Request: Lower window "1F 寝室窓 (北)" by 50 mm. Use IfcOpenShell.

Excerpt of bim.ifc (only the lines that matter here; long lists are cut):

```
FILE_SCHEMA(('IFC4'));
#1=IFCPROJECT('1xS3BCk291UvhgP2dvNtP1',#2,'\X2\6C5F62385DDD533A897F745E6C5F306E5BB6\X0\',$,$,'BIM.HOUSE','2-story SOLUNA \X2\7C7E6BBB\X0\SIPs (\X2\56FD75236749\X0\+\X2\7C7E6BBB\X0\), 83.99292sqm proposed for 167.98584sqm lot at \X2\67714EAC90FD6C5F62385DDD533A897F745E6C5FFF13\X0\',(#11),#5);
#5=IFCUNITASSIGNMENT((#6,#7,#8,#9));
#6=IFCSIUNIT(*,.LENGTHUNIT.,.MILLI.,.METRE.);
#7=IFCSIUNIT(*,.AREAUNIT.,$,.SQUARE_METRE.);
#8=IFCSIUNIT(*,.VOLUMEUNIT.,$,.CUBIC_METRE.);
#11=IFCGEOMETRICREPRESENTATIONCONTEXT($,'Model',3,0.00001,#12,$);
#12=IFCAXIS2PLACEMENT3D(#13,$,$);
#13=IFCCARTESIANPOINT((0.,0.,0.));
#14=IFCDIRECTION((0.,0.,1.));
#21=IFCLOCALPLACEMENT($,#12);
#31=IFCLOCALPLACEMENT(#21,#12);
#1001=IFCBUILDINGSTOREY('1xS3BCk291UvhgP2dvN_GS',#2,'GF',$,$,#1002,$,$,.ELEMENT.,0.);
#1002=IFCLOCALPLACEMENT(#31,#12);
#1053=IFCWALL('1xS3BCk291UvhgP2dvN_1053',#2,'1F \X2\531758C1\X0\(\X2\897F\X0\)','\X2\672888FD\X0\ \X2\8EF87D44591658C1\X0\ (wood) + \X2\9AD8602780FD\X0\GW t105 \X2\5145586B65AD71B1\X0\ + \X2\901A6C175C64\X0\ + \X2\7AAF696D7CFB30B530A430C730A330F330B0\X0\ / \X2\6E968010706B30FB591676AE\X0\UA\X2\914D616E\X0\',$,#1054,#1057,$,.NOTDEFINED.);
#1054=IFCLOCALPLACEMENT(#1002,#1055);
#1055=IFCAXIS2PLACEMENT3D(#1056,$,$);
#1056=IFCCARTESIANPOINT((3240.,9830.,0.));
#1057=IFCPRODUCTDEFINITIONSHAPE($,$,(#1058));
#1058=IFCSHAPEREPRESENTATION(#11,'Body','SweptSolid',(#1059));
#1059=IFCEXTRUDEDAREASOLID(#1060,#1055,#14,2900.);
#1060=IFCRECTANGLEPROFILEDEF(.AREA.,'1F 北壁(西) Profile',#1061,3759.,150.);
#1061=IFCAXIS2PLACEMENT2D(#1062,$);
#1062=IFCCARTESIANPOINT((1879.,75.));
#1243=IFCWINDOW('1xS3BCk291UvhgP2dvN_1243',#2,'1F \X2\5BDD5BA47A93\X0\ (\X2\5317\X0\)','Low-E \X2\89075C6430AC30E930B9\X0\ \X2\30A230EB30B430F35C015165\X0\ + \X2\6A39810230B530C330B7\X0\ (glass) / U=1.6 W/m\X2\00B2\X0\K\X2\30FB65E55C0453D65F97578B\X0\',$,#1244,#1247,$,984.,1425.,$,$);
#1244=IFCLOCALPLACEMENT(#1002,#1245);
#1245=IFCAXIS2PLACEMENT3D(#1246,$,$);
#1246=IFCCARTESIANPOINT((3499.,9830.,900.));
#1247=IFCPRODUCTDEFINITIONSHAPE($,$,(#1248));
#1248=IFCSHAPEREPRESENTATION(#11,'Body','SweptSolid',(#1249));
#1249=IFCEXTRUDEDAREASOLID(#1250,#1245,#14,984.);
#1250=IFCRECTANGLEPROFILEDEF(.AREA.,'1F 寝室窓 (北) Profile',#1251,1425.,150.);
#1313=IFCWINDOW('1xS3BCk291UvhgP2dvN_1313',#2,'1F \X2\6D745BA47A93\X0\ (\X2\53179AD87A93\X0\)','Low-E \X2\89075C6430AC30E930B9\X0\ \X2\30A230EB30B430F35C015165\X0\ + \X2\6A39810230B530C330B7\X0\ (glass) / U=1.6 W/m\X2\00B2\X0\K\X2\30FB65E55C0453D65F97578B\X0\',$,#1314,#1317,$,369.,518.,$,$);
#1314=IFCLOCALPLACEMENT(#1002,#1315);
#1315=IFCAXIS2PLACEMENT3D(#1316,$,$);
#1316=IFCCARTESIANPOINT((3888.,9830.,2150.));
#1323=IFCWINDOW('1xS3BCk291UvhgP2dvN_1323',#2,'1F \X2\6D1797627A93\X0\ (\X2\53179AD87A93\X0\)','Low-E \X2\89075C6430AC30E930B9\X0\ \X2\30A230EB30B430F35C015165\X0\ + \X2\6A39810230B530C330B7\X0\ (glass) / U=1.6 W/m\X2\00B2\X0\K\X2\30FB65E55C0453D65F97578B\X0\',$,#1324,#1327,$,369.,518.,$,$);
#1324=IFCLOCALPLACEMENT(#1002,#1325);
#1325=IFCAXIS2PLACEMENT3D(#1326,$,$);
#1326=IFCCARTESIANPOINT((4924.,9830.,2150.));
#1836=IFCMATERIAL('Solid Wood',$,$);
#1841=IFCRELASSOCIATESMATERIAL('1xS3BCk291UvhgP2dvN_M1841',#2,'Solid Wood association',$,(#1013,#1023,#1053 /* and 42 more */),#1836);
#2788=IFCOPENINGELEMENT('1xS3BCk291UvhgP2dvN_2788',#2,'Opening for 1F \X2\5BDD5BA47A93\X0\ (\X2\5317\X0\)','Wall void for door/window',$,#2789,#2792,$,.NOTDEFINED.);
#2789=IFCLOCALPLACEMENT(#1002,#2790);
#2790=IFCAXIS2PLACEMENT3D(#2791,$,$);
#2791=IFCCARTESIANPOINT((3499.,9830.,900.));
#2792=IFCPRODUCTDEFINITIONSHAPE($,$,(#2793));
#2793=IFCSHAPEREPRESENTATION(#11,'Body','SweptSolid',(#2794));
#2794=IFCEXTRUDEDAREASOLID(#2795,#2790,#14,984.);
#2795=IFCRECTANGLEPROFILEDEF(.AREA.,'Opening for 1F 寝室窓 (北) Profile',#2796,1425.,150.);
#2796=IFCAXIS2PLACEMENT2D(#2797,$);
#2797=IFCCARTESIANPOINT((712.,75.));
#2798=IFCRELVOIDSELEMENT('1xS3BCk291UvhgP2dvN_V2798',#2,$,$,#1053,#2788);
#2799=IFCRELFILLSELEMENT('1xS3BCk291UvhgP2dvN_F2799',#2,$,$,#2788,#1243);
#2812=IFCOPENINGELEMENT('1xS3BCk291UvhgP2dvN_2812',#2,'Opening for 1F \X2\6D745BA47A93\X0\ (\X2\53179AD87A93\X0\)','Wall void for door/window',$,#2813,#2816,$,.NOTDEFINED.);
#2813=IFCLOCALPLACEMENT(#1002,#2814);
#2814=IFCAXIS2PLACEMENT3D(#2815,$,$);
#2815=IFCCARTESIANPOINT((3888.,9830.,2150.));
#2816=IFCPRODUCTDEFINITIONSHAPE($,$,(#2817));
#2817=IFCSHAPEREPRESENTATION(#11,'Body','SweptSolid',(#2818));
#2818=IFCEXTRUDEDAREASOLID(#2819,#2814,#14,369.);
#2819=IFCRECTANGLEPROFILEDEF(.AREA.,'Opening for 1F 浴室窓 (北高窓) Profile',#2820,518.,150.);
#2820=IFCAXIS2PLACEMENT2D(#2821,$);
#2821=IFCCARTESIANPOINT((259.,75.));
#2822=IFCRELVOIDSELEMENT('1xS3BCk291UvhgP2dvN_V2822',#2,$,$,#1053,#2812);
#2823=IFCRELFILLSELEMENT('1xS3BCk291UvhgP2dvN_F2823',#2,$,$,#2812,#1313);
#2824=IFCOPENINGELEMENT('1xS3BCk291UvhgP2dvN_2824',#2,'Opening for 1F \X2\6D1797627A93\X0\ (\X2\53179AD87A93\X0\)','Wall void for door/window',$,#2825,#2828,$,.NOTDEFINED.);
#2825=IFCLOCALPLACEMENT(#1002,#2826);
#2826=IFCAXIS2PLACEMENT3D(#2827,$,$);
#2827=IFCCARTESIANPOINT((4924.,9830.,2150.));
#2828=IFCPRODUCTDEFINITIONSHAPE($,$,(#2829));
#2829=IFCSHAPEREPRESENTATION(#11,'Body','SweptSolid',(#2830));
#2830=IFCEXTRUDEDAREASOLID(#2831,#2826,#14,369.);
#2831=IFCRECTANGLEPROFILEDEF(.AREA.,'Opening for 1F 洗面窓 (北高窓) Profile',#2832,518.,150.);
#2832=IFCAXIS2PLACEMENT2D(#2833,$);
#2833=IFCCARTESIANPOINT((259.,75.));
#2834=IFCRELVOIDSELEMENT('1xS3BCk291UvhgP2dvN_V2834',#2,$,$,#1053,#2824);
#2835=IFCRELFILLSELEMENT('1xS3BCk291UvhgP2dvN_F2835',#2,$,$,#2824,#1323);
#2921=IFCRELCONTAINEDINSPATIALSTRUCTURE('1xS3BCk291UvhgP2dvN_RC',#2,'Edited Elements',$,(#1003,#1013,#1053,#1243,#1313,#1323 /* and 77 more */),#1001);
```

```python
import numpy as np
import ifcopenshell
import ifcopenshell.api.geometry
import ifcopenshell.util.placement
import ifcopenshell.util.unit

model = ifcopenshell.open("bim.ifc")
unit_scale = ifcopenshell.util.unit.calculate_unit_scale(model)

window = model.by_id(1243)
opening = window.FillsVoids[0].RelatingOpeningElement
dz = -0.05 / unit_scale

shift = np.array([0.0, 0.0, dz])
# The window is not placed relative to its opening, so move both.
for product in (opening, window):
    matrix = ifcopenshell.util.placement.get_local_placement(product.ObjectPlacement)
    matrix[:3, 3] += shift
    ifcopenshell.api.geometry.edit_object_placement(model, product=product, matrix=matrix, is_si=False)

print(f"moved by {dz * unit_scale:+.3f} m")

model.write("bim_rev.ifc")
```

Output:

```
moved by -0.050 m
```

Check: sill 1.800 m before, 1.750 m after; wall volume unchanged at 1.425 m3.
